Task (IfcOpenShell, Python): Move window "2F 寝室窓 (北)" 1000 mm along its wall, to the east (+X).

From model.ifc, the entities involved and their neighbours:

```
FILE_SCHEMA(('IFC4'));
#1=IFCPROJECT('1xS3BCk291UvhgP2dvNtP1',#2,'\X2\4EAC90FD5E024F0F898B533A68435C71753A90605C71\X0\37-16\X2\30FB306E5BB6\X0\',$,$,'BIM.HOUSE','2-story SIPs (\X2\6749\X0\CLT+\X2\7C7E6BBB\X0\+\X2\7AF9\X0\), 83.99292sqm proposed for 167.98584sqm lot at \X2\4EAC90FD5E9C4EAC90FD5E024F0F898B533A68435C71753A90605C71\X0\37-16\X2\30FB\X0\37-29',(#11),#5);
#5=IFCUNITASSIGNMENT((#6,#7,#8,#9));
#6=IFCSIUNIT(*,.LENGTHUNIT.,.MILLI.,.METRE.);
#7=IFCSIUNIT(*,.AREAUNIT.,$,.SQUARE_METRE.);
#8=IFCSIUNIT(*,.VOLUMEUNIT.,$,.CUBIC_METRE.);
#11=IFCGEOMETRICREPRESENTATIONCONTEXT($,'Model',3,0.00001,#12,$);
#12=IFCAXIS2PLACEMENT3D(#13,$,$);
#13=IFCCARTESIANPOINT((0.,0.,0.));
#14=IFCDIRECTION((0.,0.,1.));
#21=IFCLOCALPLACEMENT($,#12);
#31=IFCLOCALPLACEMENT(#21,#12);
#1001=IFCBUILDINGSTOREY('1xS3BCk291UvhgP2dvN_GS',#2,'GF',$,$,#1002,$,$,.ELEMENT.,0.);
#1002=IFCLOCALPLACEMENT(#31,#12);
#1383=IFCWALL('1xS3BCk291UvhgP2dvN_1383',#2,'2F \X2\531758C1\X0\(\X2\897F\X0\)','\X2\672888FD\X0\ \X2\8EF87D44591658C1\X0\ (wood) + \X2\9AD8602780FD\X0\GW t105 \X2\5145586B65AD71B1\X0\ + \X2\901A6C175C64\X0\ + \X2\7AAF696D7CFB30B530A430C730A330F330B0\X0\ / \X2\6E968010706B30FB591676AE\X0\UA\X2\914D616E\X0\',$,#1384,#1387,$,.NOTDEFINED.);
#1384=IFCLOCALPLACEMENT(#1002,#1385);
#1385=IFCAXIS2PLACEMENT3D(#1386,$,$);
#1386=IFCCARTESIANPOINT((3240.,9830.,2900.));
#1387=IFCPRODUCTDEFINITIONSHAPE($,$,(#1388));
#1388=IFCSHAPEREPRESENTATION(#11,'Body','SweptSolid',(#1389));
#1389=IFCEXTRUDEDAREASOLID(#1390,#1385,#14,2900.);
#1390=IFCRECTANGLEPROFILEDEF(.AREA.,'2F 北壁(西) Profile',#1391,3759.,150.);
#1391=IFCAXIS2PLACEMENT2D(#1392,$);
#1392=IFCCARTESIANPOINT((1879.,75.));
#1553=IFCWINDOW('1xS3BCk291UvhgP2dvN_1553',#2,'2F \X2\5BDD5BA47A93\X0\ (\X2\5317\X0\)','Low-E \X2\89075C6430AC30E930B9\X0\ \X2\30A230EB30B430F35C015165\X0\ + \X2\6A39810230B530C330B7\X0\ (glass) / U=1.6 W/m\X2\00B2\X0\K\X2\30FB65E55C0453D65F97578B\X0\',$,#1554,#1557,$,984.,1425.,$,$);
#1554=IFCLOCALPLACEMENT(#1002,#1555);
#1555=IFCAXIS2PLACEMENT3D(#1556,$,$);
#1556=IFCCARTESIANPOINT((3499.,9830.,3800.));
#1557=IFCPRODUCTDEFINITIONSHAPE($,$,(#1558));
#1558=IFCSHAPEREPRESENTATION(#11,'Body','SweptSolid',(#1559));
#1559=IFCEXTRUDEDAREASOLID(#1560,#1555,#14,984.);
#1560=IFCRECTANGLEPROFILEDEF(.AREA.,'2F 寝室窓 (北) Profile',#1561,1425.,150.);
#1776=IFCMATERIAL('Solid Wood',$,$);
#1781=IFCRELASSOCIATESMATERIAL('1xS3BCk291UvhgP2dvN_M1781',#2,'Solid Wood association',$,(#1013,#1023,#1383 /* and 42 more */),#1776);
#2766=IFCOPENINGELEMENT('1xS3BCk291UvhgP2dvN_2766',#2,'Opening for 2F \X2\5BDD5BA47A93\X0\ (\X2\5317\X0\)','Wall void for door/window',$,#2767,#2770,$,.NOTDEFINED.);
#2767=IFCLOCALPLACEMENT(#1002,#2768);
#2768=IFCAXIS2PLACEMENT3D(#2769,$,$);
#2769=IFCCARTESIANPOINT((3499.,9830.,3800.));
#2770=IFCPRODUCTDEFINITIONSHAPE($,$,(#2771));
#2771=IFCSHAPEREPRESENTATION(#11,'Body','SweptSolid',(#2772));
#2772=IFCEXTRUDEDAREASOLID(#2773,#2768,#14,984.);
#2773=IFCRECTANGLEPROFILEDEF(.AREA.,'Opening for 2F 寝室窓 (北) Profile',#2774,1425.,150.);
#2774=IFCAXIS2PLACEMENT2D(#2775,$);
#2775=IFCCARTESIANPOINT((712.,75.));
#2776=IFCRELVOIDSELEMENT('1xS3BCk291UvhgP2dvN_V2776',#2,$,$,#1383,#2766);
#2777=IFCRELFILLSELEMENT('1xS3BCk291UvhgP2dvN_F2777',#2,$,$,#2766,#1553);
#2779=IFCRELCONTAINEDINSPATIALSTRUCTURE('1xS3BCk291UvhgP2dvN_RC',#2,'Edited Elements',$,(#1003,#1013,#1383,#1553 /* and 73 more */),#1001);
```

```python
import ifcopenshell
import ifcopenshell.api.geometry
import ifcopenshell.util.placement

model = ifcopenshell.open("model.ifc")

window = model.by_id(1553)
opening = window.FillsVoids[0].RelatingOpeningElement
wall = opening.VoidsElements[0].RelatingBuildingElement

wall_matrix = ifcopenshell.util.placement.get_local_placement(wall.ObjectPlacement)
shift = wall_matrix[:3, 0] * 1000.0
before = ifcopenshell.util.placement.get_local_placement(window.ObjectPlacement)[:3, 3].copy()

# The window is not placed relative to its opening, so move both.
for product in (opening, window):
    matrix = ifcopenshell.util.placement.get_local_placement(product.ObjectPlacement)
    matrix[:3, 3] += shift
    ifcopenshell.api.geometry.edit_object_placement(model, product=product, matrix=matrix, is_si=False)

after = ifcopenshell.util.placement.get_local_placement(window.ObjectPlacement)[:3, 3]
print("window moved by", (after - before).round(3) + 0.0)

model.write("model_edited.ifc")
```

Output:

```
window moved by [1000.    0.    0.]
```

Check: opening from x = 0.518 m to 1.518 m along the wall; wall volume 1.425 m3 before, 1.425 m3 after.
